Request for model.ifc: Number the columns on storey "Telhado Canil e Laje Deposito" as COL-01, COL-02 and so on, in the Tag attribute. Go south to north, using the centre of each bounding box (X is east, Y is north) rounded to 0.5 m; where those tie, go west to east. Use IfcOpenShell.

First a look at what the model holds.

```python
import ifcopenshell
import ifcopenshell.util.element
import ifcopenshell.util.placement

model = ifcopenshell.open("model.ifc")
print(model.schema)
storey = next(s for s in model.by_type("IfcBuildingStorey") if s.Name == "Telhado Canil e Laje Deposito")
columns = [e for e in ifcopenshell.util.element.get_decomposition(storey) if e.is_a("IfcColumn")]
for e in sorted(columns, key=lambda e: e.id()):
    origin = ifcopenshell.util.placement.get_local_placement(e.ObjectPlacement)[:3, 3]
    print(e.id(), e.Tag, e.Name, origin.round(2) + 0.0, sep=" | ")
```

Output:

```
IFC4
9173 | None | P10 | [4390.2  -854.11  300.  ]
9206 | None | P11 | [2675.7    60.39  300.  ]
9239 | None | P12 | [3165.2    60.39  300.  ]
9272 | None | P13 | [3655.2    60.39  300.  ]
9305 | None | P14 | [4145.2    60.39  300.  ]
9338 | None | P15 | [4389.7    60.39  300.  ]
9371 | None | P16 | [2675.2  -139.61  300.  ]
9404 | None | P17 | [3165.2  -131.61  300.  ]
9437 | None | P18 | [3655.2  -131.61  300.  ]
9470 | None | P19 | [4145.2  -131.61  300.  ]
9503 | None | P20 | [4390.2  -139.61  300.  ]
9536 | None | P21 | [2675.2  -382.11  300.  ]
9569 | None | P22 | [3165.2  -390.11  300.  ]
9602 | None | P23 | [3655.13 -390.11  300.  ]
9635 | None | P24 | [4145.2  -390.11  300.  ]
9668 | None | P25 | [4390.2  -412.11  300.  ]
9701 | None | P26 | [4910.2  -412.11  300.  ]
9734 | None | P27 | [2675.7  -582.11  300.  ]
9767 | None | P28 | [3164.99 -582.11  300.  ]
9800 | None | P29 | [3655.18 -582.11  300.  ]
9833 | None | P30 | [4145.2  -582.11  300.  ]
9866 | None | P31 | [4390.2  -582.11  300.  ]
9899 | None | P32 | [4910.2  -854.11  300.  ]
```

```python
import ifcopenshell
import ifcopenshell.geom
import ifcopenshell.util.element
import ifcopenshell.util.shape

model = ifcopenshell.open("model.ifc")
settings = ifcopenshell.geom.settings()
settings.set("use-world-coords", True)


def centre(element):
    shape = ifcopenshell.geom.create_shape(settings, element)
    return ifcopenshell.util.shape.get_bbox_centroid(shape.geometry)


storey = next(s for s in model.by_type("IfcBuildingStorey") if s.Name == "Telhado Canil e Laje Deposito")
columns = [e for e in ifcopenshell.util.element.get_decomposition(storey) if e.is_a("IfcColumn")]

# Insertion points can sit at a corner or the storey origin, so sort by the geometry (in metres).
centres = {e: centre(e) for e in columns}
columns.sort(key=lambda e: (round(centres[e][1] / 0.5), centres[e][0]))

for i, e in enumerate(columns, start=1):
    number = f"COL-{i:02d}"
    e.Tag = number
    print(e.id(), number)

model.write("model_rev.ifc")
```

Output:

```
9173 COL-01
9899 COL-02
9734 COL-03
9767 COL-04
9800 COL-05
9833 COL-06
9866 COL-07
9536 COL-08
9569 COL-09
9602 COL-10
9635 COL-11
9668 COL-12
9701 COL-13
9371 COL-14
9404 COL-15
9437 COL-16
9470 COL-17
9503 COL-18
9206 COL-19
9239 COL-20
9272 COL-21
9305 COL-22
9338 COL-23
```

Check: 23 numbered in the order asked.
